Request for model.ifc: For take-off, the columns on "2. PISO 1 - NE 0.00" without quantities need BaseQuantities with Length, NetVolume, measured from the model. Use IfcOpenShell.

First a look at what the model holds.

```python
import ifcopenshell
import ifcopenshell.util.element
import ifcopenshell.util.unit

model = ifcopenshell.open("model.ifc")
print(model.schema)
for unit_type in ("LENGTHUNIT", "AREAUNIT", "VOLUMEUNIT"):
    print(unit_type, ifcopenshell.util.unit.calculate_unit_scale(model, unit_type))
storey = next(s for s in model.by_type("IfcBuildingStorey") if s.Name == "2. PISO 1 - NE 0.00")
columns = [e for e in ifcopenshell.util.element.get_decomposition(storey) if e.is_a("IfcColumn")]
for e in sorted(columns, key=lambda e: e.id()):
    print(e.id(), e.is_a(), e.Name, list(ifcopenshell.util.element.get_psets(e, qtos_only=True)), sep=" | ")
```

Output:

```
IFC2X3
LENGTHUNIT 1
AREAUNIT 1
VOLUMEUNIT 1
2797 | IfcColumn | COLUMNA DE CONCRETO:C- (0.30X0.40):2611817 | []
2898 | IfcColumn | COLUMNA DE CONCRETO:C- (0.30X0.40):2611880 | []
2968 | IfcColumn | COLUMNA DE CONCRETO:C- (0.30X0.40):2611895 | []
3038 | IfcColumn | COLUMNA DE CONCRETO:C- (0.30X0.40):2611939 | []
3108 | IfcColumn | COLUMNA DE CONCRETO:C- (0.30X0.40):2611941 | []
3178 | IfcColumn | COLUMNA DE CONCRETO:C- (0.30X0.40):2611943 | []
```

```python
import ifcopenshell
import ifcopenshell.api.pset
import ifcopenshell.geom
import ifcopenshell.util.element
import ifcopenshell.util.shape
import ifcopenshell.util.unit

model = ifcopenshell.open("model.ifc")
unit_scale = ifcopenshell.util.unit.calculate_unit_scale(model)
volume_scale = ifcopenshell.util.unit.calculate_unit_scale(model, "VOLUMEUNIT")
settings = ifcopenshell.geom.settings()

storey = next(s for s in model.by_type("IfcBuildingStorey") if s.Name == "2. PISO 1 - NE 0.00")
columns = [e for e in ifcopenshell.util.element.get_decomposition(storey) if e.is_a("IfcColumn")]

for e in sorted(columns, key=lambda e: e.id()):
    if ifcopenshell.util.element.get_psets(e, qtos_only=True, should_inherit=False):
        continue
    # Geometry comes back in metres, in the element's own axes.
    shape = ifcopenshell.geom.create_shape(settings, e)
    values = {
        "Length": ifcopenshell.util.shape.get_z(shape.geometry) / unit_scale,
        "NetVolume": ifcopenshell.util.shape.get_volume(shape.geometry) / volume_scale,
    }
    qto = ifcopenshell.api.pset.add_qto(model, product=e, name="BaseQuantities")
    ifcopenshell.api.pset.edit_qto(model, qto=qto, properties=values)
    print(e.id(), {k: round(v, 3) for k, v in values.items()})

model.write("model_updated.ifc")
```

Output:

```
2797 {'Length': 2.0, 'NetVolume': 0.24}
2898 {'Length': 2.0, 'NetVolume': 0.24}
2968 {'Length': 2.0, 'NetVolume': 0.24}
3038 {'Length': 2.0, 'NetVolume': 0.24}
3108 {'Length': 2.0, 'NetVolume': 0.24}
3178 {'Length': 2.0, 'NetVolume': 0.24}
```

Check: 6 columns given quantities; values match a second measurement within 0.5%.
